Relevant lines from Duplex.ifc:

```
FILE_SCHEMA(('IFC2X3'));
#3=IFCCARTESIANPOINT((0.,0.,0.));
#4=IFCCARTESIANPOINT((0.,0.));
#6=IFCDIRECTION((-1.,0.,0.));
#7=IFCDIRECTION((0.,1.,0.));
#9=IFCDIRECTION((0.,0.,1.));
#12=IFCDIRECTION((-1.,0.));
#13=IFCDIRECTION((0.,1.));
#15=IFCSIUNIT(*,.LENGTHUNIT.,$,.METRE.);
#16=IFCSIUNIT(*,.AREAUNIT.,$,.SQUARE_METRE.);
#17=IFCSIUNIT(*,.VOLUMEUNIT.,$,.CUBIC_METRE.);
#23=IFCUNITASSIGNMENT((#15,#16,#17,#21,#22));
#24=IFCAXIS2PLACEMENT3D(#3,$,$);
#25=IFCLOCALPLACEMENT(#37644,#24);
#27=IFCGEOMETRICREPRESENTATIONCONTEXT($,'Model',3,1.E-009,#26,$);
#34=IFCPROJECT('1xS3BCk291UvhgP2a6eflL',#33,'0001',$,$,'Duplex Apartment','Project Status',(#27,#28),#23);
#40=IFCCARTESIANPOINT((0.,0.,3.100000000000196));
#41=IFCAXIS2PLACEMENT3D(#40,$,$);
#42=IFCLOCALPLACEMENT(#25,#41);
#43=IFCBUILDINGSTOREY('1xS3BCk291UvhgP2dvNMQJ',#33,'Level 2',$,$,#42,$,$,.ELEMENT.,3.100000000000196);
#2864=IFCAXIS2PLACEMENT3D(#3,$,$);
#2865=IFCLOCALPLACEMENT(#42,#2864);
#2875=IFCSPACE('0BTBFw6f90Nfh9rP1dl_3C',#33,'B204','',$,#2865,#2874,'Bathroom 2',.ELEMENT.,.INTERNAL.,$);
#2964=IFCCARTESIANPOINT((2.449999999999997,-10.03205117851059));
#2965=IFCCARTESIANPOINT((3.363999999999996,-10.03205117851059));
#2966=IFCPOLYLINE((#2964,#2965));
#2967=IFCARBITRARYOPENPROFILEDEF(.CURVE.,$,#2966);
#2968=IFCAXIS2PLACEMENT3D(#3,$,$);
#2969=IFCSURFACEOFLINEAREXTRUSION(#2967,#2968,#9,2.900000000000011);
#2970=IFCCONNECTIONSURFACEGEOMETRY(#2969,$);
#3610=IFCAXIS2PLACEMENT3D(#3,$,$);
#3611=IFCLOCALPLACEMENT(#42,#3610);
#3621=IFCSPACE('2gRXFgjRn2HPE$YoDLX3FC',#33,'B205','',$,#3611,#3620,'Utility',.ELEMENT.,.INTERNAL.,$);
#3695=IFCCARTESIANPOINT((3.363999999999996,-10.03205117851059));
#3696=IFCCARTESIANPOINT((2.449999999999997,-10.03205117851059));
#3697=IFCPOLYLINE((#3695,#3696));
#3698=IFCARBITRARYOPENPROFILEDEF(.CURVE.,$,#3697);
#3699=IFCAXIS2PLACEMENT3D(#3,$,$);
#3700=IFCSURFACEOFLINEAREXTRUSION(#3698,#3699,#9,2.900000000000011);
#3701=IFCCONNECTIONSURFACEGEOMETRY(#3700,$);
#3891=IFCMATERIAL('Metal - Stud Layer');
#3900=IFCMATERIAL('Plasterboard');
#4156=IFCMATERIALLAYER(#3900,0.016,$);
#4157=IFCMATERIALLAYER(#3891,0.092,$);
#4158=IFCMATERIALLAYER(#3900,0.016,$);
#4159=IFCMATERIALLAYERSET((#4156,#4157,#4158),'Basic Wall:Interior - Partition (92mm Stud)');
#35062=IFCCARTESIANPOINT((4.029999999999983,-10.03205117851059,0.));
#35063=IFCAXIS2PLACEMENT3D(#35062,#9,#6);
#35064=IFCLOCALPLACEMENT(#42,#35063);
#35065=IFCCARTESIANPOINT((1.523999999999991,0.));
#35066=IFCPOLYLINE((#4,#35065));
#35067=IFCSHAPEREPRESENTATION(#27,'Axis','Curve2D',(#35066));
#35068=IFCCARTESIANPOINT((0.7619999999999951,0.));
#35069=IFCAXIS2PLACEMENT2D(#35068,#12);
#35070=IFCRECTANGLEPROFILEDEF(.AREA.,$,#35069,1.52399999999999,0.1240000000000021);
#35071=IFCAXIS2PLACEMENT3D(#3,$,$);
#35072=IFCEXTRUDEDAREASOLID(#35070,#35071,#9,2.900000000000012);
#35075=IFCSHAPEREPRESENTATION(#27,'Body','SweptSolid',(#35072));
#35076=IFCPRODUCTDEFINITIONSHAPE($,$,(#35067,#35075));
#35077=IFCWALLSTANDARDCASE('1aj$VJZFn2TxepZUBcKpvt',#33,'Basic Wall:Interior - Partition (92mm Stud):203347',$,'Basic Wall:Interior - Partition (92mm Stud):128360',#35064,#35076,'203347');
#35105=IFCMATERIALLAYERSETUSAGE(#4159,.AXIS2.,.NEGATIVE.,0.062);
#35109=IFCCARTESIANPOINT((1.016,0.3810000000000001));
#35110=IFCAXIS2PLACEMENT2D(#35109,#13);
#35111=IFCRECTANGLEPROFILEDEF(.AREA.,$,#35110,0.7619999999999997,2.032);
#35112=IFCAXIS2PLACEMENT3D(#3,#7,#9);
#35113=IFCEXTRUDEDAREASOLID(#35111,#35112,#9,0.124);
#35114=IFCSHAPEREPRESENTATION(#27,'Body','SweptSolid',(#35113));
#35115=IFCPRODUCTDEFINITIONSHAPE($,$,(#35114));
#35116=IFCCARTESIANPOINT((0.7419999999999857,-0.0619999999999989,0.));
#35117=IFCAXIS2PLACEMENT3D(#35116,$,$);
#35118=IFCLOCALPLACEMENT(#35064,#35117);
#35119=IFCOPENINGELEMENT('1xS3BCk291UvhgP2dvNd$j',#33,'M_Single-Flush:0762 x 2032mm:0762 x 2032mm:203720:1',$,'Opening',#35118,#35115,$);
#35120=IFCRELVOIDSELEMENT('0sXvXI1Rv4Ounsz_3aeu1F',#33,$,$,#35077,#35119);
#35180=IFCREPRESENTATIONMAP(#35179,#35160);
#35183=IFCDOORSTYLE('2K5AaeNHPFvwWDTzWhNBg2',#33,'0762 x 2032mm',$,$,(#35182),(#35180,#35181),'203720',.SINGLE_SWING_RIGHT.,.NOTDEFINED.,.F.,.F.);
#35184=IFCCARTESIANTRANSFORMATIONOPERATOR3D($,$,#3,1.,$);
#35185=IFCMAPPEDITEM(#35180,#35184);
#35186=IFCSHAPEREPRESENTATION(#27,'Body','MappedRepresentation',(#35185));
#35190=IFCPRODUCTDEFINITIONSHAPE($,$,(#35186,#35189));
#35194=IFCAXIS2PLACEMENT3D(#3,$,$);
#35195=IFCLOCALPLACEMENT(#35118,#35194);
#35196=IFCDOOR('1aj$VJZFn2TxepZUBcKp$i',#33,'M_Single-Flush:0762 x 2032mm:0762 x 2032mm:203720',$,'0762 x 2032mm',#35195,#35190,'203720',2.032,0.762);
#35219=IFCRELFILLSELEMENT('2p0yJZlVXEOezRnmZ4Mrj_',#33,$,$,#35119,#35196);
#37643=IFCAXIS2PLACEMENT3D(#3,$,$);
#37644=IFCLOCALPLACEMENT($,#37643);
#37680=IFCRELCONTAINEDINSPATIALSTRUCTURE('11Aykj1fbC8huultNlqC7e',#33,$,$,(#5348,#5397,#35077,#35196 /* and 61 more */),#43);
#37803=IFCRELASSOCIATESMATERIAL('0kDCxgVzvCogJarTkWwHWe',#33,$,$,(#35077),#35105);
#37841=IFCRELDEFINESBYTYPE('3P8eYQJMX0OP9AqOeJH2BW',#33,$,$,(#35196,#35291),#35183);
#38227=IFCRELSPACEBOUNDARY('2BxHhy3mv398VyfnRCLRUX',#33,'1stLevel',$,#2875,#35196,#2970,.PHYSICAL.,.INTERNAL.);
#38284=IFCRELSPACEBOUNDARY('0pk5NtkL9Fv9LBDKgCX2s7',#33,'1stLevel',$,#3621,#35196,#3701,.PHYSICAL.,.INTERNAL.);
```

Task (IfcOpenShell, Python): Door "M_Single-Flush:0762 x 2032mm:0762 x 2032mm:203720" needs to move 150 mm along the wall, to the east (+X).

```python
import numpy as np
import ifcopenshell
import ifcopenshell.api.geometry
import ifcopenshell.util.placement
import ifcopenshell.util.unit

model = ifcopenshell.open("Duplex.ifc")
unit_scale = ifcopenshell.util.unit.calculate_unit_scale(model)

door = model.by_id(35196)
opening = door.FillsVoids[0].RelatingOpeningElement
wall = opening.VoidsElements[0].RelatingBuildingElement

wall_matrix = ifcopenshell.util.placement.get_local_placement(wall.ObjectPlacement)
shift = wall_matrix[:3, 0] * -0.15 / unit_scale
before = ifcopenshell.util.placement.get_local_placement(door.ObjectPlacement)[:3, 3].copy()

# The door is placed relative to its opening, so it follows when the opening moves.
matrix = ifcopenshell.util.placement.get_local_placement(opening.ObjectPlacement)
matrix[:3, 3] += shift
ifcopenshell.api.geometry.edit_object_placement(
    model, product=opening, matrix=matrix, is_si=False, should_transform_children=True
)

# Space boundary surfaces are stored in each space's coordinates; move them too.
for rel in door.ProvidesBoundaries:
    if not rel.ConnectionGeometry:
        continue
    surface = rel.ConnectionGeometry.SurfaceOnRelatingElement
    space_matrix = ifcopenshell.util.placement.get_local_placement(rel.RelatingSpace.ObjectPlacement)
    point = np.array(surface.Position.Location.Coordinates) + space_matrix[:3, :3].T @ shift
    surface.Position = model.createIfcAxis2Placement3D(
        model.createIfcCartesianPoint(point.tolist()), surface.Position.Axis, surface.Position.RefDirection
    )

after = ifcopenshell.util.placement.get_local_placement(door.ObjectPlacement)[:3, 3]
print("door moved by", (after - before).round(3) + 0.0)

model.write("Duplex_rev.ifc")
```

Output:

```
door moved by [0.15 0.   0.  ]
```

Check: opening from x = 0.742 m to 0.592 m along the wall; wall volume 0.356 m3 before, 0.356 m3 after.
